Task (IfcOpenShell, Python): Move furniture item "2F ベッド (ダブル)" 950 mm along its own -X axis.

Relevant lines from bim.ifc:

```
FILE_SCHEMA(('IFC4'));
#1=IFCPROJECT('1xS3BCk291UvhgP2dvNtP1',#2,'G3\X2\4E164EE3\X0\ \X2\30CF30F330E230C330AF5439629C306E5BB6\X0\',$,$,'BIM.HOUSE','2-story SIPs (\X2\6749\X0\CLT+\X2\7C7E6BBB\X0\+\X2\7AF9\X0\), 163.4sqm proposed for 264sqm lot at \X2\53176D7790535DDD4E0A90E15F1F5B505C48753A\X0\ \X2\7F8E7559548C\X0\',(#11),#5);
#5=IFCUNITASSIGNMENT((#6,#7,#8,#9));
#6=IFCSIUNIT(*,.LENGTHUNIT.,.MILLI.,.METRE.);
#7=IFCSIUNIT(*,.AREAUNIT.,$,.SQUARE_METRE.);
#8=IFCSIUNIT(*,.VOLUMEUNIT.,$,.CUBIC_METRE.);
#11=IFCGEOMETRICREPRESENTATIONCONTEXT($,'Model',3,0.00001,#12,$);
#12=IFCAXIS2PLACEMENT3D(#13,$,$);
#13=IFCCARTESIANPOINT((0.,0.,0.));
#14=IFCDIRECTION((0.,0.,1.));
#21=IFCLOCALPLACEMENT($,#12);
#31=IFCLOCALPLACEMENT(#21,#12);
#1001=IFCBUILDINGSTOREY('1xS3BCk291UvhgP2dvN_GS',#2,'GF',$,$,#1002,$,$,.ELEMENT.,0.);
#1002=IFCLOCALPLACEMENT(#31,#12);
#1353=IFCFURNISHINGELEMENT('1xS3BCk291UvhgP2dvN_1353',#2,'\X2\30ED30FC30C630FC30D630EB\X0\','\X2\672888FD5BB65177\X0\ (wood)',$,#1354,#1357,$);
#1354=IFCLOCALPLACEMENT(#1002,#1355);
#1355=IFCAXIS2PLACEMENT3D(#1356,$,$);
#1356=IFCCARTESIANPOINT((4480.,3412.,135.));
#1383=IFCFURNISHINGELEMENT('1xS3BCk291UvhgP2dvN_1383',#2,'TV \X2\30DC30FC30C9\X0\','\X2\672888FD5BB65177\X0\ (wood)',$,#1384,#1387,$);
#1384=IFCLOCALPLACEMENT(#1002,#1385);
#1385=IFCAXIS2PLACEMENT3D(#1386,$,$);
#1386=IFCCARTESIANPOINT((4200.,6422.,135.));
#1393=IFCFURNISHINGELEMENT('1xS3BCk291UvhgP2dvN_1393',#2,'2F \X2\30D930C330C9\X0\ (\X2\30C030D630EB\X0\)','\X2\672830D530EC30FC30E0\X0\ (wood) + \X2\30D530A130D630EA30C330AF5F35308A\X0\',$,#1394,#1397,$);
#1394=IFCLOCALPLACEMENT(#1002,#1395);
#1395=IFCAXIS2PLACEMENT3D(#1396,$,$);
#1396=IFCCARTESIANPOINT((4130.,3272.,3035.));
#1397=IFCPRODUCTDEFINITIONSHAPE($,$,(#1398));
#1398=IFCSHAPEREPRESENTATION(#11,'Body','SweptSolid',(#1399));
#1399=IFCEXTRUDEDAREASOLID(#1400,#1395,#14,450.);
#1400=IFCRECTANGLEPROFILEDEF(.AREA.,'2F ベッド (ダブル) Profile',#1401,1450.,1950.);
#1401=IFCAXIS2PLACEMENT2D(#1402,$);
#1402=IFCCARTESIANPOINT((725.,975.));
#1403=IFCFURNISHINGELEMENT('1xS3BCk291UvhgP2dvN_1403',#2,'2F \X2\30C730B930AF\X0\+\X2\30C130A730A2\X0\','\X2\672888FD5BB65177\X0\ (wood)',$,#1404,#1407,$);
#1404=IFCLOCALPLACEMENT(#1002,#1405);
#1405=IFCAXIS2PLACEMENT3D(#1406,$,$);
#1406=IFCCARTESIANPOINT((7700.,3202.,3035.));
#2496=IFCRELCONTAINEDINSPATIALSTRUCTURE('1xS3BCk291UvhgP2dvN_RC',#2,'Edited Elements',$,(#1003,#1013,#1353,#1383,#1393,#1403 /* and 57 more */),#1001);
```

```python
import ifcopenshell
import ifcopenshell.api.geometry
import ifcopenshell.util.placement

model = ifcopenshell.open("bim.ifc")

item = model.by_id(1393)
matrix = ifcopenshell.util.placement.get_local_placement(item.ObjectPlacement)
matrix[:3, 3] -= matrix[:3, 0] * 950.0
ifcopenshell.api.geometry.edit_object_placement(model, product=item, matrix=matrix, is_si=False)

print(ifcopenshell.util.placement.get_local_placement(item.ObjectPlacement).round(3) + 0.0)

model.write("bim-out.ifc")
```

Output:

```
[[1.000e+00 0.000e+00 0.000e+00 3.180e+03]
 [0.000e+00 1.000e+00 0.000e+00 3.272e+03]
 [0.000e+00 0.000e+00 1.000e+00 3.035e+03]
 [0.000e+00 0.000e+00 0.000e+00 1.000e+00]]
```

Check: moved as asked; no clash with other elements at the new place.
